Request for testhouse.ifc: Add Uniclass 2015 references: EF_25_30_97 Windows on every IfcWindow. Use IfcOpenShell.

First a look at what the model holds.

```python
import ifcopenshell

model = ifcopenshell.open("testhouse.ifc")
print(model.schema)
print("classifications:", [c.Name for c in model.by_type("IfcClassification")])
for ifc_class in ("IfcDoor", "IfcRoof", "IfcStair", "IfcWall", "IfcWindow"):
    print(ifc_class, len(model.by_type(ifc_class)))
```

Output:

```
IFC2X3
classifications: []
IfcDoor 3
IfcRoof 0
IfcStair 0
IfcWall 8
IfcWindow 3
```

```python
import ifcopenshell
import ifcopenshell.api.classification

model = ifcopenshell.open("testhouse.ifc")

# IFC2X3 requires Source and Edition and has no link from the project to the system.
system = model.create_entity("IfcClassification", Source="NBS", Edition="2015", Name="Uniclass 2015")

codes = {
    "IfcWindow": ("EF_25_30_97", "Windows"),
}
for ifc_class, (code, name) in codes.items():
    products = model.by_type(ifc_class)
    ifcopenshell.api.classification.add_reference(
        model, products=products, classification=system, identification=code, name=name
    )
    print(code, len(products))

model.write("testhouse_edited.ifc")
```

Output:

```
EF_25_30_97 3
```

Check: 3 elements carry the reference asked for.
